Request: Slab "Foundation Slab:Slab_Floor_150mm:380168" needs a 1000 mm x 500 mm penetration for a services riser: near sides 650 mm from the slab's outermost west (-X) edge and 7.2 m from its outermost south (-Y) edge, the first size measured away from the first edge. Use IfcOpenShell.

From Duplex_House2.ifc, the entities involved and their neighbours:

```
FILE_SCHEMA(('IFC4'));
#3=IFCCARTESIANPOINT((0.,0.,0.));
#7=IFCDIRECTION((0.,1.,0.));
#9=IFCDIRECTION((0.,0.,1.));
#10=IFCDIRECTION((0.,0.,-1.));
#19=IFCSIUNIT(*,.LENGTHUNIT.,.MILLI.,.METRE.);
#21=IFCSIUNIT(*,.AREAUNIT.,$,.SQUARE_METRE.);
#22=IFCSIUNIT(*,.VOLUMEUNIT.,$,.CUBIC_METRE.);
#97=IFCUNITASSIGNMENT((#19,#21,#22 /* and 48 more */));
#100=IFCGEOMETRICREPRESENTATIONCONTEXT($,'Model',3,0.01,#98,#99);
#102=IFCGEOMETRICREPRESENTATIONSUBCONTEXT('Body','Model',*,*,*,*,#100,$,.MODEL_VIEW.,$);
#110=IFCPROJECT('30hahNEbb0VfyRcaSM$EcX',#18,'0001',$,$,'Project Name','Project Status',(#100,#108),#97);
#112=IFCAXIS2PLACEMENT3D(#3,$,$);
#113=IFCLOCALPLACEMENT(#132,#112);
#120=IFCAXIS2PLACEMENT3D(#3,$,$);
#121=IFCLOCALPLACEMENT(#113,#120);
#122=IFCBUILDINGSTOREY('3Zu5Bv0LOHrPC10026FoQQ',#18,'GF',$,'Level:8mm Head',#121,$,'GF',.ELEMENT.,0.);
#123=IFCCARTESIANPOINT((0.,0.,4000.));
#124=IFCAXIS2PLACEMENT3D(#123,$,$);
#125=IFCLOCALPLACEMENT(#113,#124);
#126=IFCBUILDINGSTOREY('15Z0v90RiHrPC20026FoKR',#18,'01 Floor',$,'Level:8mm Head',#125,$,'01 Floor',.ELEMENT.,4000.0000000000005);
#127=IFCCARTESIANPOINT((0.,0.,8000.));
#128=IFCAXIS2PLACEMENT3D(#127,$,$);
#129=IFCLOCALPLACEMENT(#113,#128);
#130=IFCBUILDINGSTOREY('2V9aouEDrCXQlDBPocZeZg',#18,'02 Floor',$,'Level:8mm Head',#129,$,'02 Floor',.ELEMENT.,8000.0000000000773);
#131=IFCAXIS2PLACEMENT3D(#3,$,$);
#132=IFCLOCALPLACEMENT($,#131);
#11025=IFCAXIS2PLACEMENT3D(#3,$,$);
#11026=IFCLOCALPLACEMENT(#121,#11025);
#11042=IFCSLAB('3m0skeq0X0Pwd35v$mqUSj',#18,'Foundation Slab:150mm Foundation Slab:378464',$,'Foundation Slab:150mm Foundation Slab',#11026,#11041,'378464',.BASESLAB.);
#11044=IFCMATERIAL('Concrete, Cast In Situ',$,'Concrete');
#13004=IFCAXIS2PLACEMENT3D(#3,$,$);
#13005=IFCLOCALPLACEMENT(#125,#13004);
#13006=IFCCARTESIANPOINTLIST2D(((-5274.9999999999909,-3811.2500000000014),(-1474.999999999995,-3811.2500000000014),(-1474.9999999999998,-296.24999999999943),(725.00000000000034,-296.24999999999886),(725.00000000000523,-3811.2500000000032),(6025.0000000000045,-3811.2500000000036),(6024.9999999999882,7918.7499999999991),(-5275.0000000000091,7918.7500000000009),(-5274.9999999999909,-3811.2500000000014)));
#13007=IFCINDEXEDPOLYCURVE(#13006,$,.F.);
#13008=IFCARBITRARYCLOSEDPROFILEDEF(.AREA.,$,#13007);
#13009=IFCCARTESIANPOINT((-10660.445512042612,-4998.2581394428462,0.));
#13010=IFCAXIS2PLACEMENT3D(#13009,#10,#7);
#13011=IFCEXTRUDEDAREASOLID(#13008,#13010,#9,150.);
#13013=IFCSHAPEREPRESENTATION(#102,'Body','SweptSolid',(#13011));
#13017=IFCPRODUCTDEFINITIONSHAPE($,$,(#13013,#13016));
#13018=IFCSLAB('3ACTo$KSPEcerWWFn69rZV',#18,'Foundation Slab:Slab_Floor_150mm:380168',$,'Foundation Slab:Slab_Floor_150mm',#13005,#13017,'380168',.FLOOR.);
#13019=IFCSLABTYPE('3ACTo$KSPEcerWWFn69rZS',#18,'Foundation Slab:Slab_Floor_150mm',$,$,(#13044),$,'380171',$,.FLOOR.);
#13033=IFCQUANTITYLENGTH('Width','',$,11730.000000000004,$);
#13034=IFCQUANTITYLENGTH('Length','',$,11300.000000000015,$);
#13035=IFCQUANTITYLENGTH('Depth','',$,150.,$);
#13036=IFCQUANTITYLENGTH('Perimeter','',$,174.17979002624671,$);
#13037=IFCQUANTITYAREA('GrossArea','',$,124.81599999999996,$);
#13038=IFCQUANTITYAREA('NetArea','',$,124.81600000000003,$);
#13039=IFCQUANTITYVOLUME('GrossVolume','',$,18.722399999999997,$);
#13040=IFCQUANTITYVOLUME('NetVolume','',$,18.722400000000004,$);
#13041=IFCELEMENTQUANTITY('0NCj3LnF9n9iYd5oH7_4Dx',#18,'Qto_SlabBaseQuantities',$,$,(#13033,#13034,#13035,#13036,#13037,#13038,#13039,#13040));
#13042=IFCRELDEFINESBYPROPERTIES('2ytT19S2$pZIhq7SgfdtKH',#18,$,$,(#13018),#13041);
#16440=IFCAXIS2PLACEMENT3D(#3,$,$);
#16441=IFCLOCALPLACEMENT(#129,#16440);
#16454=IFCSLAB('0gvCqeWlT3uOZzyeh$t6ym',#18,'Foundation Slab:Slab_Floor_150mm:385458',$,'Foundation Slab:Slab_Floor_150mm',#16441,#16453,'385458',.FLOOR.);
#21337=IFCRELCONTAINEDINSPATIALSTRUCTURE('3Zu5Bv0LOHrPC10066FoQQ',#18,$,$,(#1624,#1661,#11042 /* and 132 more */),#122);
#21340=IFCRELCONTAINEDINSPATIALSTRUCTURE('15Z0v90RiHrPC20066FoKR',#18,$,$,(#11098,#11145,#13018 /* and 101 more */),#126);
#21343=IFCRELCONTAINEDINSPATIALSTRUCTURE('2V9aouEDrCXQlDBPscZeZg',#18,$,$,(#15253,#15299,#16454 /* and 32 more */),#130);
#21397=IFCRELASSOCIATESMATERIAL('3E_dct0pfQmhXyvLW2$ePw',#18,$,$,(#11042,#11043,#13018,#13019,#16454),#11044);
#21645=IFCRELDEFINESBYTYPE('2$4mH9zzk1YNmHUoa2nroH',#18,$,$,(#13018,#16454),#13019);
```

```python
import numpy as np
import ifcopenshell
import ifcopenshell.api.feature
import ifcopenshell.api.geometry
import ifcopenshell.api.pset
import ifcopenshell.api.root
import ifcopenshell.geom
import ifcopenshell.util.element
import ifcopenshell.util.placement
import ifcopenshell.util.representation
import ifcopenshell.util.shape
import ifcopenshell.util.unit

model = ifcopenshell.open("Duplex_House2.ifc")
unit_scale = ifcopenshell.util.unit.calculate_unit_scale(model)
area_scale = ifcopenshell.util.unit.calculate_unit_scale(model, "AREAUNIT")
volume_scale = ifcopenshell.util.unit.calculate_unit_scale(model, "VOLUMEUNIT")
settings = ifcopenshell.geom.settings()


def volume(element):
    """Net volume in cubic metres, openings subtracted."""
    shape = ifcopenshell.geom.create_shape(settings, element)
    return ifcopenshell.util.shape.get_volume(shape.geometry)


slab = model.by_id(13018)
before = volume(slab)

# Extent in the slab's own axes, in metres. The edges named are its -X and -Y sides.
slab_shape = ifcopenshell.geom.create_shape(settings, slab)
vertices = ifcopenshell.util.shape.get_vertices(slab_shape.geometry)
x_min, y_min, bottom = vertices.min(axis=0)
top = vertices[:, 2].max()

opening = ifcopenshell.api.root.create_entity(model, ifc_class="IfcOpeningElement", name="Services riser opening", predefined_type="OPENING")
context = ifcopenshell.util.representation.get_context(model, "Model", "Body", "MODEL_VIEW")
width, depth = 1, 0.5
outline = [(0.0, 0.0), (width, 0.0), (width, depth), (0.0, depth), (0.0, 0.0)]
# Overshoot both faces by 50 mm so the cut is clean.
shape = ifcopenshell.api.geometry.add_slab_representation(
    model, context=context, depth=top - bottom + 0.1, polyline=outline
)
ifcopenshell.api.geometry.assign_representation(model, product=opening, representation=shape)

matrix = ifcopenshell.util.placement.get_local_placement(slab.ObjectPlacement)
matrix[:, 3] = matrix @ np.append(np.array([x_min + 0.65, y_min + 7.2, bottom - 0.05]) / unit_scale, 1.0)
ifcopenshell.api.geometry.edit_object_placement(model, product=opening, matrix=matrix, is_si=False)
ifcopenshell.api.feature.add_feature(model, feature=opening, element=slab)

after = volume(slab)

# Update the slab's stored quantities.
qto = model.by_id(ifcopenshell.util.element.get_pset(slab, "Qto_SlabBaseQuantities", should_inherit=False)["id"])
ifcopenshell.api.pset.edit_qto(model, qto=qto, properties={
    "NetArea": after / (top - bottom) / area_scale,
    "NetVolume": after / volume_scale,
})

print(f"slab volume {before:.3f} -> {after:.3f} m3")

model.write("Duplex_House2-out.ifc")
```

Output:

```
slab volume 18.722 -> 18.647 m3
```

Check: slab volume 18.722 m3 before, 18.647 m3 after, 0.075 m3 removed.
